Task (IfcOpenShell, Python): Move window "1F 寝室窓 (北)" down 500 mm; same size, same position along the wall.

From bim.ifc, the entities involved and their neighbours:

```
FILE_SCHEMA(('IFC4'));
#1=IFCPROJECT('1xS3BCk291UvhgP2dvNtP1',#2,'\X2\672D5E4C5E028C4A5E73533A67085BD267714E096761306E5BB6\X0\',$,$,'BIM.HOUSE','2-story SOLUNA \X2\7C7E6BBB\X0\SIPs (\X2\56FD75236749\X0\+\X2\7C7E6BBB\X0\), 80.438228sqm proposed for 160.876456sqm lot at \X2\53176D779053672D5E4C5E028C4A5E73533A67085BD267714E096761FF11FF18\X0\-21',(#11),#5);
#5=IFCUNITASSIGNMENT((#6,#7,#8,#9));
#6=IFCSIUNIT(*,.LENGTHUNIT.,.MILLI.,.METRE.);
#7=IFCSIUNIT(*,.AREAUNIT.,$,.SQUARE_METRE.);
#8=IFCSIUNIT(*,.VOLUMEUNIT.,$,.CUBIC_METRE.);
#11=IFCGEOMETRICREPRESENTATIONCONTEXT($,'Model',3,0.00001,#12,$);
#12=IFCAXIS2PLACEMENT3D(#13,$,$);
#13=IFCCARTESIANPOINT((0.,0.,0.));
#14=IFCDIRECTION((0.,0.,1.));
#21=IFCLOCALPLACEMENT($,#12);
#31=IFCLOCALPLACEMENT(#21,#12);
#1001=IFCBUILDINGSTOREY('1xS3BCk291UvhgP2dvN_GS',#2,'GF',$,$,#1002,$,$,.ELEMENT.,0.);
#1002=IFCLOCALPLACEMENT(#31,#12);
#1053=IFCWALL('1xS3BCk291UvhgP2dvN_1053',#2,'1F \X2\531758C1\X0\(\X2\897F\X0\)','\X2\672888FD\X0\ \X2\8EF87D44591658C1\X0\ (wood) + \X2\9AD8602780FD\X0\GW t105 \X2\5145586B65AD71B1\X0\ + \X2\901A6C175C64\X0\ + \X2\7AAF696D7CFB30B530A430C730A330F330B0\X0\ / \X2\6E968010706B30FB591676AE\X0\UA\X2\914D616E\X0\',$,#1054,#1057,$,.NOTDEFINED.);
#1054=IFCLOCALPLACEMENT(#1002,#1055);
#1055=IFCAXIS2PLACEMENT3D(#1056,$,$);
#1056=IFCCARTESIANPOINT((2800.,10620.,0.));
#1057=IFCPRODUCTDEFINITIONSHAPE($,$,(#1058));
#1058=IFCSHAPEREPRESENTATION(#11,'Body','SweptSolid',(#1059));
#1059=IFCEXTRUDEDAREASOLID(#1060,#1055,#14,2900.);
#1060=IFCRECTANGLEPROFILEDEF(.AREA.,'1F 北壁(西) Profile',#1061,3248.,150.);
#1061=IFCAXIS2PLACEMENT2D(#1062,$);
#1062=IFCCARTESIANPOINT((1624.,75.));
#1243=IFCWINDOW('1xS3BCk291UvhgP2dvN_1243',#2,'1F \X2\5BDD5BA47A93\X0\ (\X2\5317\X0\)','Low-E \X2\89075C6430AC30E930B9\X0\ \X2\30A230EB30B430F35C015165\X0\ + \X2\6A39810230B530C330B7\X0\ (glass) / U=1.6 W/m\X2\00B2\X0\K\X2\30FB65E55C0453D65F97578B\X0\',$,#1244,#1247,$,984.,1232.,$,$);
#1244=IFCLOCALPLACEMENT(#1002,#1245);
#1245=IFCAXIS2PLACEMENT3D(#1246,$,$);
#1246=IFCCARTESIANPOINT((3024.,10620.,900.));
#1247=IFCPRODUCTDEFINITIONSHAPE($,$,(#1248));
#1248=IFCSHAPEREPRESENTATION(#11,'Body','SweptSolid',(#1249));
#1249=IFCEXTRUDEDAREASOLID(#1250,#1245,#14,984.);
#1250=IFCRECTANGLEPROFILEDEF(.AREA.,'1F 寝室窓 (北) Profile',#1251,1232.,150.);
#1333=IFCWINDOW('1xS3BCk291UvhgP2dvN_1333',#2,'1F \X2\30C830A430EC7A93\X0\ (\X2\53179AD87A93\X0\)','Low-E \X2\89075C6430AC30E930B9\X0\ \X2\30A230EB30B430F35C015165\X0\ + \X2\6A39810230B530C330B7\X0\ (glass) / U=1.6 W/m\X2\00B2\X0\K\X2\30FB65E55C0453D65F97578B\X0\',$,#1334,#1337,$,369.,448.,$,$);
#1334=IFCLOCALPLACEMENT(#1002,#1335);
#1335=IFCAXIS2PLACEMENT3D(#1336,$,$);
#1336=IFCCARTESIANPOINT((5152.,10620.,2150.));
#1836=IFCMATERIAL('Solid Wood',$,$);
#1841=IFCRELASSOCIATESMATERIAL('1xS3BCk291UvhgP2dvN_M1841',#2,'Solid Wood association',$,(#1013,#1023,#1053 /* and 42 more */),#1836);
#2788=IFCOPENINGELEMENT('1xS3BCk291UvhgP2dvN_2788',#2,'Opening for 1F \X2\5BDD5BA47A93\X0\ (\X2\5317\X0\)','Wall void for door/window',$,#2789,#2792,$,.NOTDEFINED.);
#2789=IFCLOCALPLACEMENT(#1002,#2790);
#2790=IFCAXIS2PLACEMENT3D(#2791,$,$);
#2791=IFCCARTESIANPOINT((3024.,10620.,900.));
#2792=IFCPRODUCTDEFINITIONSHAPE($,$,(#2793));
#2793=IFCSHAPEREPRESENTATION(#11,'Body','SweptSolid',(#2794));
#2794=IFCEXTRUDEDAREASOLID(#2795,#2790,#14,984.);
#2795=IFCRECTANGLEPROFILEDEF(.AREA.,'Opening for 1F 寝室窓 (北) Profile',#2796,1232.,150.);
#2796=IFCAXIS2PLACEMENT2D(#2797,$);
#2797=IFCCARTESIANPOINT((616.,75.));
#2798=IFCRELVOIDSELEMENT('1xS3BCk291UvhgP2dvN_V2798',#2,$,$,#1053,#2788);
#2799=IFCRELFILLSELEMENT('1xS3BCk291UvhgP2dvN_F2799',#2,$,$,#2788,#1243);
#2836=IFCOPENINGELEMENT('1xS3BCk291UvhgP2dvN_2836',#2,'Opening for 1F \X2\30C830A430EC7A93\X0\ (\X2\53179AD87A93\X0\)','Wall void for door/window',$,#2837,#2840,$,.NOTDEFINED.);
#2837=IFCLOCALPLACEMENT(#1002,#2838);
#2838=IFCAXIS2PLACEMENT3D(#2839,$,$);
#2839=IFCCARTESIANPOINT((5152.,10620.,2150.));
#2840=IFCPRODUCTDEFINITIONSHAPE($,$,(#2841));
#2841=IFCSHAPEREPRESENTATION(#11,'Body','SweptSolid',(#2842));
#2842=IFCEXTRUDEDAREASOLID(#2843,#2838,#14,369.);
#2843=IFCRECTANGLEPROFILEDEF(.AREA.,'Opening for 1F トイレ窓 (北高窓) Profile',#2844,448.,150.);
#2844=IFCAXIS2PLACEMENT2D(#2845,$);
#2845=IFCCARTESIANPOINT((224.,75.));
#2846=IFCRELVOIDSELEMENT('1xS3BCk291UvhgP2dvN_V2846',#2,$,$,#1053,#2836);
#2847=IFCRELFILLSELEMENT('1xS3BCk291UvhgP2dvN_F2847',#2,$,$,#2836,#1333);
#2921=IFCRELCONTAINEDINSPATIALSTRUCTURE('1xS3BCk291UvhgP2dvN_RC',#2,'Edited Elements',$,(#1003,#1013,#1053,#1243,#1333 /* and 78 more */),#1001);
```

```python
import numpy as np
import ifcopenshell
import ifcopenshell.api.geometry
import ifcopenshell.util.placement
import ifcopenshell.util.unit

model = ifcopenshell.open("bim.ifc")
unit_scale = ifcopenshell.util.unit.calculate_unit_scale(model)

window = model.by_guid("1xS3BCk291UvhgP2dvN_1243")
opening = window.FillsVoids[0].RelatingOpeningElement
dz = -500.0

shift = np.array([0.0, 0.0, dz])
# The window is not placed relative to its opening, so move both.
for product in (opening, window):
    matrix = ifcopenshell.util.placement.get_local_placement(product.ObjectPlacement)
    matrix[:3, 3] += shift
    ifcopenshell.api.geometry.edit_object_placement(model, product=product, matrix=matrix, is_si=False)

print(f"moved by {dz * unit_scale:+.3f} m")

model.write("bim_v2.ifc")
```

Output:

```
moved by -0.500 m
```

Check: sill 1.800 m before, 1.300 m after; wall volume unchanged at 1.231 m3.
